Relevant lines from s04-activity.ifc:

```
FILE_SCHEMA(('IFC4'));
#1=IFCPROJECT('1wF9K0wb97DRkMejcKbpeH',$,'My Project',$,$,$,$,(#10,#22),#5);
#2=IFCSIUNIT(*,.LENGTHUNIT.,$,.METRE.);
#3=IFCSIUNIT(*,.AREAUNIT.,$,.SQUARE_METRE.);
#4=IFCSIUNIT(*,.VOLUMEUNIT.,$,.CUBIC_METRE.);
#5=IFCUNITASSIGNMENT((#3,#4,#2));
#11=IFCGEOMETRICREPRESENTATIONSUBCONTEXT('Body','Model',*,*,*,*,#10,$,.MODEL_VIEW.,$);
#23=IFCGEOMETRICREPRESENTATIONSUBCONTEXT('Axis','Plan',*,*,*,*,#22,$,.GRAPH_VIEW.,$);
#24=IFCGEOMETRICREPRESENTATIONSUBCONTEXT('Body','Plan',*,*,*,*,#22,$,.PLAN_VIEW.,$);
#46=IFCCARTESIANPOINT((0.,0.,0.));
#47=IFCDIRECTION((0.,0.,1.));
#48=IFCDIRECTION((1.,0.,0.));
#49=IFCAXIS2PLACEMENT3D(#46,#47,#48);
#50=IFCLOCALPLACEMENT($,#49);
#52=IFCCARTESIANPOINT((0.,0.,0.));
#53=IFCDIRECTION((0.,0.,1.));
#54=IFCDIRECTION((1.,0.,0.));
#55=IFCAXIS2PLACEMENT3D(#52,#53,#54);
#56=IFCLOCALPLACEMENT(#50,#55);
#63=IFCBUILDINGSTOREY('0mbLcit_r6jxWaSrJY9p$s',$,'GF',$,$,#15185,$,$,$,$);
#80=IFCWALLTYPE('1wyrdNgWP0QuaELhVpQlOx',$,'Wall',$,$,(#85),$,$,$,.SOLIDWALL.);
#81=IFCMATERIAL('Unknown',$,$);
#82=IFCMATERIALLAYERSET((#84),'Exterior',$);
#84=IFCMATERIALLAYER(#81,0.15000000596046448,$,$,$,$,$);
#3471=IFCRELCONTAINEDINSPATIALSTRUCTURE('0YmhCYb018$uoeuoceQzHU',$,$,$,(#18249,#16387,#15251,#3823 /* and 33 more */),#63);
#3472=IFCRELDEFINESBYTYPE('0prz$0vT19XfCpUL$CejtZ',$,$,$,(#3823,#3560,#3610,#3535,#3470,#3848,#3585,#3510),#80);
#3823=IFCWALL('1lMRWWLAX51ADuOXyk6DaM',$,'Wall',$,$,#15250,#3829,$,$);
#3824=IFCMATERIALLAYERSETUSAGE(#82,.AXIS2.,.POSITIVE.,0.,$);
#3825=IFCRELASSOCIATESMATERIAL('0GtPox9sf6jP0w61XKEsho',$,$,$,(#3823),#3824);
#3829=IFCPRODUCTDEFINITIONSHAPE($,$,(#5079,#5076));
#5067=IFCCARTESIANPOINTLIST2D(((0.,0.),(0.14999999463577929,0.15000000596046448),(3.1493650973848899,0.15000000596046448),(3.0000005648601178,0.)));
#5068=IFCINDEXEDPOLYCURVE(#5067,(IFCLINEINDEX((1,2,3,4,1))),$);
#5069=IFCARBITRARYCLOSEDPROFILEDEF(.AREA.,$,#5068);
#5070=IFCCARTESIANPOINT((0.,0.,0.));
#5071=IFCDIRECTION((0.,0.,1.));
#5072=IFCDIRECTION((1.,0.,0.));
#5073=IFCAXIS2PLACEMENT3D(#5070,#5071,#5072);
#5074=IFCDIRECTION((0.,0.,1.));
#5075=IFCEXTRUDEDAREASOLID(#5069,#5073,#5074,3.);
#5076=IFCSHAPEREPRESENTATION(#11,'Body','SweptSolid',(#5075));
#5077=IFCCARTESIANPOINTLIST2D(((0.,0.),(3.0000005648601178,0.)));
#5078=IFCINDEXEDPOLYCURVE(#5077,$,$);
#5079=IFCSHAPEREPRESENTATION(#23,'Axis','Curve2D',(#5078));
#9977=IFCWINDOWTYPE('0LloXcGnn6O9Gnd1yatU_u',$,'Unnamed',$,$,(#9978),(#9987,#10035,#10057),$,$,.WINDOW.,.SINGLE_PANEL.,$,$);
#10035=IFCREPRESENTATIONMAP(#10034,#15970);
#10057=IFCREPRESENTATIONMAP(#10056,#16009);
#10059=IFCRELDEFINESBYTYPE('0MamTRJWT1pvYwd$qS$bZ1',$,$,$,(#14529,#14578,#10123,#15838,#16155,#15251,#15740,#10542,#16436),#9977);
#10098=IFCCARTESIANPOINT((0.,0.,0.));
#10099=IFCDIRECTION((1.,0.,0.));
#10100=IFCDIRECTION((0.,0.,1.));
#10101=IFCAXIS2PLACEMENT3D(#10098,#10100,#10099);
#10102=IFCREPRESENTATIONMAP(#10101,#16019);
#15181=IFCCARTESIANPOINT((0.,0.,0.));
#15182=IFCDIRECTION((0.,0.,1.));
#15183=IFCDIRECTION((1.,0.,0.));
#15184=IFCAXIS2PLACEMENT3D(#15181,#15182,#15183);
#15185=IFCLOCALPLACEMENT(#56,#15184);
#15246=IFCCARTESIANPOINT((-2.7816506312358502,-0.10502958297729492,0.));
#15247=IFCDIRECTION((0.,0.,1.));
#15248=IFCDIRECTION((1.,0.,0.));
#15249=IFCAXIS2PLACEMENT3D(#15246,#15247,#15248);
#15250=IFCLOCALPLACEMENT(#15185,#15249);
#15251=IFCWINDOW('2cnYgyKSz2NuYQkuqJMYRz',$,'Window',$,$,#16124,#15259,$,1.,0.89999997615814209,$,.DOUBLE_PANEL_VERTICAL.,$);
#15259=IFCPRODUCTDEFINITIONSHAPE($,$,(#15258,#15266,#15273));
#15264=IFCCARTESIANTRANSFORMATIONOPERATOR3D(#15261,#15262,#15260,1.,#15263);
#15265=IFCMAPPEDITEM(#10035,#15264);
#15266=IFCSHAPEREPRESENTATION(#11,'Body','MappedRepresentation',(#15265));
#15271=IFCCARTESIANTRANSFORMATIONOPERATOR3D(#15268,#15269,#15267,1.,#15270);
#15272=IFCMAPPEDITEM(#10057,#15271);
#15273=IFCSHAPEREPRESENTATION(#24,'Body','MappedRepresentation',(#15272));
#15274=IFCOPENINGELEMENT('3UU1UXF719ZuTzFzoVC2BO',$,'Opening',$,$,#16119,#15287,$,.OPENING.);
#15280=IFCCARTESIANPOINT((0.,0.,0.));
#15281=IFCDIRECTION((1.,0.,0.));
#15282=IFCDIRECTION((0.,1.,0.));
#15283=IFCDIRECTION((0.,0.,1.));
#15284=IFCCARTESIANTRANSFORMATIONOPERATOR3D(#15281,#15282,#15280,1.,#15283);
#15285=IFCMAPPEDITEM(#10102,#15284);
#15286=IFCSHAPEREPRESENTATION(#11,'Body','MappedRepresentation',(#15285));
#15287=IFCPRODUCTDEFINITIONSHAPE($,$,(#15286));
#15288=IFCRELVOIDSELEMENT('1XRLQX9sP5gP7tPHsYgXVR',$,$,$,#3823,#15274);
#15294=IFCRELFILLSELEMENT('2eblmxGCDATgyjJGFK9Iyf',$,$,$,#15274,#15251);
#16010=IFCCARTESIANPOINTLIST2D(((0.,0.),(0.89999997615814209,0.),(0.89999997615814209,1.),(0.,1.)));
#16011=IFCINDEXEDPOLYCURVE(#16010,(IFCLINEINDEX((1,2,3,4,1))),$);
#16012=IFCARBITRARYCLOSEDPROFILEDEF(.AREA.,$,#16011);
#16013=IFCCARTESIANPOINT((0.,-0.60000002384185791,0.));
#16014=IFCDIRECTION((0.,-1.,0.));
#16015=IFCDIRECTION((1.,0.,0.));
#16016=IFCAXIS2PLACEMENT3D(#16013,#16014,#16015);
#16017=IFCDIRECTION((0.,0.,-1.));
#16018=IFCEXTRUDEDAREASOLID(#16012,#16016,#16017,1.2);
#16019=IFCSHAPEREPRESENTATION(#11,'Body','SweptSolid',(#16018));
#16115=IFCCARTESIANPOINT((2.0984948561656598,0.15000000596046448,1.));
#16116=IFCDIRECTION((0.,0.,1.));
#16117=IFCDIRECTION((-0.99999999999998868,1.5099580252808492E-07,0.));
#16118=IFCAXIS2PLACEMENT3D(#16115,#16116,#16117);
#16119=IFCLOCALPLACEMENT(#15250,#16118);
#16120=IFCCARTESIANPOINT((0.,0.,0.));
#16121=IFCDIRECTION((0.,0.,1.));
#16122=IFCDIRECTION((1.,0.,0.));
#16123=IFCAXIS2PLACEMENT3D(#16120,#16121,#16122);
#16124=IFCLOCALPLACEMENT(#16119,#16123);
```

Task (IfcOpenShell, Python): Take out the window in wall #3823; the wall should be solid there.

```python
import ifcopenshell
import ifcopenshell.api.feature
import ifcopenshell.api.root
import ifcopenshell.geom
import ifcopenshell.util.shape

model = ifcopenshell.open("s04-activity.ifc")
settings = ifcopenshell.geom.settings()


def volume(element):
    """Net volume in cubic metres, openings subtracted."""
    shape = ifcopenshell.geom.create_shape(settings, element)
    return ifcopenshell.util.shape.get_volume(shape.geometry)


window = model.by_guid("2cnYgyKSz2NuYQkuqJMYRz")
opening = window.FillsVoids[0].RelatingOpeningElement
wall = opening.VoidsElements[0].RelatingBuildingElement
before = volume(wall)

ifcopenshell.api.root.remove_product(model, product=window)
ifcopenshell.api.feature.remove_feature(model, feature=opening)

after = volume(wall)

print(f"wall volume {before:.3f} -> {after:.3f} m3")

model.write("s04-activity_rev.ifc")
```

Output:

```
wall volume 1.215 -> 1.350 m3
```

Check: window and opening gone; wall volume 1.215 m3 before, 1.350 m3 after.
